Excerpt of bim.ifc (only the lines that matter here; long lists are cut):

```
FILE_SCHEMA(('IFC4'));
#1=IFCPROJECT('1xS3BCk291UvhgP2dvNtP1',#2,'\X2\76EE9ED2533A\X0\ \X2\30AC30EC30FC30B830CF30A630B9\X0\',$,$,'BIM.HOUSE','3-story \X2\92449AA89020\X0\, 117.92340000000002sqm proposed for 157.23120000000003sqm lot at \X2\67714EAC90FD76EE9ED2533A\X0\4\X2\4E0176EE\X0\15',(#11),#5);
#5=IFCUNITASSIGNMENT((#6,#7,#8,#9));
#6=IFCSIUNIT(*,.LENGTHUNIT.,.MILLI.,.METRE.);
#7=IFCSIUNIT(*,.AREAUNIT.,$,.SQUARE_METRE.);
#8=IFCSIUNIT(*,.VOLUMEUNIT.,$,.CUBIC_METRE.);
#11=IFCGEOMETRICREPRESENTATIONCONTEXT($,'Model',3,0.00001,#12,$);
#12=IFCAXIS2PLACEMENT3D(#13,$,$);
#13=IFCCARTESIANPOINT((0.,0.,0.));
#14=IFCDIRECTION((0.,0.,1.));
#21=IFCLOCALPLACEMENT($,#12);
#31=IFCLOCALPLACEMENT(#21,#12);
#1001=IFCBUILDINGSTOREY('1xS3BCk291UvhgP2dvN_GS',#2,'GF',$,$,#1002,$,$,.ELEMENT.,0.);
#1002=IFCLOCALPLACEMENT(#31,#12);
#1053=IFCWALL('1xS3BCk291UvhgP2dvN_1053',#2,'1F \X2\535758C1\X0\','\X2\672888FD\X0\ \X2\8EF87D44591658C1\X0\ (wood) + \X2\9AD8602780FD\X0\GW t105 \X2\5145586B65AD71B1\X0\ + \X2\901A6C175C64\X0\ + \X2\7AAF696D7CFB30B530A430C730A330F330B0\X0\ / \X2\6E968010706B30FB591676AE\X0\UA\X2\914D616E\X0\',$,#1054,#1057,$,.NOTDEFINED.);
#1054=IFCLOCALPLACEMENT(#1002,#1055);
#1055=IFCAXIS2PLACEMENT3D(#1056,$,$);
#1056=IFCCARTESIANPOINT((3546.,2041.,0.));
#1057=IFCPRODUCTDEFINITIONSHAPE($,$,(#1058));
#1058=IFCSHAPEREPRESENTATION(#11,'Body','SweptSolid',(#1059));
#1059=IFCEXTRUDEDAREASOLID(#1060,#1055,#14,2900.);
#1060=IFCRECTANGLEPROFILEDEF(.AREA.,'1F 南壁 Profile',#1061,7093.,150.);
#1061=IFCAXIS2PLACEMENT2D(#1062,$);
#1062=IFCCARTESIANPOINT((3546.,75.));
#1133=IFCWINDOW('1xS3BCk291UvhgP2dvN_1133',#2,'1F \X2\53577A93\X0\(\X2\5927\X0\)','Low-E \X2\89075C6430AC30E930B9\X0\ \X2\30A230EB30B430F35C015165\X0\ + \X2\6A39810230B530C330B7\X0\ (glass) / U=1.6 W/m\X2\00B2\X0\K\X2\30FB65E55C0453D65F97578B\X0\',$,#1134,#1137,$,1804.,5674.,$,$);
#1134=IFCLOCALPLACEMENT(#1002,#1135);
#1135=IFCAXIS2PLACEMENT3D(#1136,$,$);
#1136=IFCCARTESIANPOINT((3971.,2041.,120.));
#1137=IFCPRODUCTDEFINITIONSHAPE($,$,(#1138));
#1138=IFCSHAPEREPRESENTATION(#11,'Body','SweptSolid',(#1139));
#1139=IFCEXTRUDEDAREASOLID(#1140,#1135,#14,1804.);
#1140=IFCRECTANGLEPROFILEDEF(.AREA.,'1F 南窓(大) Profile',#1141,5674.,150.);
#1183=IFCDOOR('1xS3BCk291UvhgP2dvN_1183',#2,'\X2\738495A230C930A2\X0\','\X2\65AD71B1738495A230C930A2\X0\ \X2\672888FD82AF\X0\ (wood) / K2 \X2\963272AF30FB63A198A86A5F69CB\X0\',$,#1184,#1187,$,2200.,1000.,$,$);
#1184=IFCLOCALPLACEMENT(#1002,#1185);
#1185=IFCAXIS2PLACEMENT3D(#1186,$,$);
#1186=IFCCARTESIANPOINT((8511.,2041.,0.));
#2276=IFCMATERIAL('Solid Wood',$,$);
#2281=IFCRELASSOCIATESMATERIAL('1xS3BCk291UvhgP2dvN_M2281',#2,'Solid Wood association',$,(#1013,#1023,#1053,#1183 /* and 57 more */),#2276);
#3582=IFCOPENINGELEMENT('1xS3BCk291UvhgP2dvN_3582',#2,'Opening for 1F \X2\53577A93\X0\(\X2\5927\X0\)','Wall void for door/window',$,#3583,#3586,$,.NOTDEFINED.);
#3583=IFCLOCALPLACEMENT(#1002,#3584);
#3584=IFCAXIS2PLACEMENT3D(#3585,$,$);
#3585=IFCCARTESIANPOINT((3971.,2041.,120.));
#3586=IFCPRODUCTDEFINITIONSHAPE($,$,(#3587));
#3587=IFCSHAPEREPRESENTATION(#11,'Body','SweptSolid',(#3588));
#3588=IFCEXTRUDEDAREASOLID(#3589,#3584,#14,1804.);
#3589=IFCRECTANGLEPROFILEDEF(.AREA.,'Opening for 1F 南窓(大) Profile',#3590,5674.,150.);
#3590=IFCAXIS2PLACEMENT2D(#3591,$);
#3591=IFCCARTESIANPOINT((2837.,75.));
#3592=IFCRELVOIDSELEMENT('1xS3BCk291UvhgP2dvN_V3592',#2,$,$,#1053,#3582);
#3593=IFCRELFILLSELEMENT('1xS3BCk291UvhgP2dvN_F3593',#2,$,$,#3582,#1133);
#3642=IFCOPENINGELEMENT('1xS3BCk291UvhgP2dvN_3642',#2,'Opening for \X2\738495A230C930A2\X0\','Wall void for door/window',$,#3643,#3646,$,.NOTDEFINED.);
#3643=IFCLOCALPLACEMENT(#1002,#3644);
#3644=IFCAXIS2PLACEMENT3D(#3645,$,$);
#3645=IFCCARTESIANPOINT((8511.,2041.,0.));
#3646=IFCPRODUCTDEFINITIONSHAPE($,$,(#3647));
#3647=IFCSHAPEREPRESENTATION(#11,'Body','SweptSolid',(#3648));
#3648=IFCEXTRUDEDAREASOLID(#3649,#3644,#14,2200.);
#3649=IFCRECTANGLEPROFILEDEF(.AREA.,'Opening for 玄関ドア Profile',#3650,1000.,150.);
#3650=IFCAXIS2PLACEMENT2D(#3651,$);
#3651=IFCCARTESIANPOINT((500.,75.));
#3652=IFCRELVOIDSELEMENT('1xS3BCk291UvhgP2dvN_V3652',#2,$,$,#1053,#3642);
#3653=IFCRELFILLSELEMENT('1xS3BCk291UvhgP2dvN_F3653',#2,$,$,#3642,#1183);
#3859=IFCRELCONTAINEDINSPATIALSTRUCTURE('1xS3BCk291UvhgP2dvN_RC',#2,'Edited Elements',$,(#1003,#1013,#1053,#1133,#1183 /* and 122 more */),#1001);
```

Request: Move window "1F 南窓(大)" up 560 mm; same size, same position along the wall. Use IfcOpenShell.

```python
import numpy as np
import ifcopenshell
import ifcopenshell.api.geometry
import ifcopenshell.util.placement
import ifcopenshell.util.unit

model = ifcopenshell.open("bim.ifc")
unit_scale = ifcopenshell.util.unit.calculate_unit_scale(model)

window = model.by_guid("1xS3BCk291UvhgP2dvN_1133")
opening = window.FillsVoids[0].RelatingOpeningElement
dz = 0.56 / unit_scale

shift = np.array([0.0, 0.0, dz])
# The window is not placed relative to its opening, so move both.
for product in (opening, window):
    matrix = ifcopenshell.util.placement.get_local_placement(product.ObjectPlacement)
    matrix[:3, 3] += shift
    ifcopenshell.api.geometry.edit_object_placement(model, product=product, matrix=matrix, is_si=False)

print(f"moved by {dz * unit_scale:+.3f} m")

model.write("bim_edited.ifc")
```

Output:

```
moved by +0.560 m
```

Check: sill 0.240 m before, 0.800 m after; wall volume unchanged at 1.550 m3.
